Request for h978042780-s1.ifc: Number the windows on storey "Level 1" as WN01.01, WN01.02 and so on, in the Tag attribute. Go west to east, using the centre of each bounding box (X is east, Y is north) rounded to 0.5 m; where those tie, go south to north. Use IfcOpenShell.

First a look at what the model holds.

```python
import ifcopenshell
import ifcopenshell.util.element
import ifcopenshell.util.placement

model = ifcopenshell.open("h978042780-s1.ifc")
print(model.schema)
storey = next(s for s in model.by_type("IfcBuildingStorey") if s.Name == "Level 1")
windows = [e for e in ifcopenshell.util.element.get_decomposition(storey) if e.is_a("IfcWindow")]
for e in sorted(windows, key=lambda e: e.id()):
    origin = ifcopenshell.util.placement.get_local_placement(e.ObjectPlacement)[:3, 3]
    print(e.id(), e.Tag, e.Name, origin.round(2) + 0.0, sep=" | ")
```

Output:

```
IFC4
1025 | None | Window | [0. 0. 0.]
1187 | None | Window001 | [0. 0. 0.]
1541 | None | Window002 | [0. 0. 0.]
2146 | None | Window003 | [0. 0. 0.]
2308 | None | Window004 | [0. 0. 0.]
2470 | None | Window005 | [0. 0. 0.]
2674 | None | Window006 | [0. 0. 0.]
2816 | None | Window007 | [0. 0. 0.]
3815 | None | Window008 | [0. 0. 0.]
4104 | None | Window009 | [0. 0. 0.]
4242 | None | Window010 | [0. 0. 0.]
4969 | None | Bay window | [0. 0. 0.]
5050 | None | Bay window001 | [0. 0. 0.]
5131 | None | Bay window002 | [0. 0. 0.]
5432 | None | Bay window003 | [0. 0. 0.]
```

```python
import ifcopenshell
import ifcopenshell.geom
import ifcopenshell.util.element
import ifcopenshell.util.shape

model = ifcopenshell.open("h978042780-s1.ifc")
settings = ifcopenshell.geom.settings()
settings.set("use-world-coords", True)


def centre(element):
    shape = ifcopenshell.geom.create_shape(settings, element)
    return ifcopenshell.util.shape.get_bbox_centroid(shape.geometry)


storey = next(s for s in model.by_type("IfcBuildingStorey") if s.Name == "Level 1")
windows = [e for e in ifcopenshell.util.element.get_decomposition(storey) if e.is_a("IfcWindow")]

# Insertion points can sit at a corner or the storey origin, so sort by the geometry (in metres).
centres = {e: centre(e) for e in windows}
windows.sort(key=lambda e: (round(centres[e][0] / 0.5), centres[e][1]))

for i, e in enumerate(windows, start=1):
    number = f"WN01.{i:02d}"
    e.Tag = number
    print(e.id(), number)

model.write("h978042780-s1_rev.ifc")
```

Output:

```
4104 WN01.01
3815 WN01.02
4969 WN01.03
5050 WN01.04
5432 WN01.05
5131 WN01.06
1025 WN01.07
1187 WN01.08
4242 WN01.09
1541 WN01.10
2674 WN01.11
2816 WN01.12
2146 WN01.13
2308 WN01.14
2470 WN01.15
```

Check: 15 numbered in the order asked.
